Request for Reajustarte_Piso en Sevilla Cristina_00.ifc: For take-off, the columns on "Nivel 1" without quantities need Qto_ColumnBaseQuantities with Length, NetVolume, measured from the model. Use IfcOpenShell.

First a look at what the model holds.

```python
import ifcopenshell
import ifcopenshell.util.element
import ifcopenshell.util.unit

model = ifcopenshell.open("Reajustarte_Piso en Sevilla Cristina_00.ifc")
print(model.schema)
for unit_type in ("LENGTHUNIT", "AREAUNIT", "VOLUMEUNIT"):
    print(unit_type, ifcopenshell.util.unit.calculate_unit_scale(model, unit_type))
storey = next(s for s in model.by_type("IfcBuildingStorey") if s.Name == "Nivel 1")
columns = [e for e in ifcopenshell.util.element.get_decomposition(storey) if e.is_a("IfcColumn")]
for e in sorted(columns, key=lambda e: e.id()):
    print(e.id(), e.is_a(), e.Name, list(ifcopenshell.util.element.get_psets(e, qtos_only=True)), sep=" | ")
```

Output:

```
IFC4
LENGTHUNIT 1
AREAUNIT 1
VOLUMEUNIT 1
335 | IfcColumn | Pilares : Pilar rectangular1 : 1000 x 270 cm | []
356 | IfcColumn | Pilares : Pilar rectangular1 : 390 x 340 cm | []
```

```python
import ifcopenshell
import ifcopenshell.api.pset
import ifcopenshell.geom
import ifcopenshell.util.element
import ifcopenshell.util.shape
import ifcopenshell.util.unit

model = ifcopenshell.open("Reajustarte_Piso en Sevilla Cristina_00.ifc")
unit_scale = ifcopenshell.util.unit.calculate_unit_scale(model)
volume_scale = ifcopenshell.util.unit.calculate_unit_scale(model, "VOLUMEUNIT")
settings = ifcopenshell.geom.settings()

storey = next(s for s in model.by_type("IfcBuildingStorey") if s.Name == "Nivel 1")
columns = [e for e in ifcopenshell.util.element.get_decomposition(storey) if e.is_a("IfcColumn")]

for e in sorted(columns, key=lambda e: e.id()):
    if ifcopenshell.util.element.get_psets(e, qtos_only=True, should_inherit=False):
        continue
    # Geometry comes back in metres, in the element's own axes.
    shape = ifcopenshell.geom.create_shape(settings, e)
    values = {
        "Length": ifcopenshell.util.shape.get_z(shape.geometry) / unit_scale,
        "NetVolume": ifcopenshell.util.shape.get_volume(shape.geometry) / volume_scale,
    }
    qto = ifcopenshell.api.pset.add_qto(model, product=e, name="Qto_ColumnBaseQuantities")
    ifcopenshell.api.pset.edit_qto(model, qto=qto, properties=values)
    print(e.id(), {k: round(v, 3) for k, v in values.items()})

model.write("Reajustarte_Piso en Sevilla Cristina_00_updated.ifc")
```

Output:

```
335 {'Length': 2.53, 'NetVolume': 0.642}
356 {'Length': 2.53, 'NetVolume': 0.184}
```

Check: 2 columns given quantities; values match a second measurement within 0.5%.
